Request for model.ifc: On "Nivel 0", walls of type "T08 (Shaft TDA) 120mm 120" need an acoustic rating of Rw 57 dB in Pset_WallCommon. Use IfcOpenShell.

First a look at what the model holds.

```python
import ifcopenshell
import ifcopenshell.util.element

model = ifcopenshell.open("model.ifc")
print(model.schema)
storey = next(s for s in model.by_type("IfcBuildingStorey") if s.Name == "Nivel 0")
walls = [e for e in ifcopenshell.util.element.get_decomposition(storey) if e.is_a("IfcWall")]
seen = {}
for e in walls:
    element_type = ifcopenshell.util.element.get_type(e)
    key = (element_type.Name if element_type != e and element_type else None, ifcopenshell.util.element.get_pset(e, "Pset_WallCommon", "AcousticRating"))
    seen[key] = seen.get(key, 0) + 1
for (name, value), count in sorted(seen.items(), key=str):
    print(count, "x", name, "|", value)
```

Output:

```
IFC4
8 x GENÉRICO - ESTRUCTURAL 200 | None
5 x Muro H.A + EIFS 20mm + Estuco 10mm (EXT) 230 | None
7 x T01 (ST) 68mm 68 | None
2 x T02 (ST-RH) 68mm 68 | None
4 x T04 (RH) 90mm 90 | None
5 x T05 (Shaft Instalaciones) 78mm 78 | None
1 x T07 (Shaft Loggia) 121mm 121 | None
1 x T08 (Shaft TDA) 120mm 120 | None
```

```python
import ifcopenshell
import ifcopenshell.api.pset
import ifcopenshell.util.element

model = ifcopenshell.open("model.ifc")

storey = next(s for s in model.by_type("IfcBuildingStorey") if s.Name == "Nivel 0")
walls = [e for e in ifcopenshell.util.element.get_decomposition(storey) if e.is_a("IfcWall")]

count = 0
for e in walls:
    element_type = ifcopenshell.util.element.get_type(e)
    if element_type in (None, e) or element_type.Name != "T08 (Shaft TDA) 120mm 120":
        continue
    # add_pset returns the element's existing set when there is one.
    pset = ifcopenshell.api.pset.add_pset(model, product=e, name="Pset_WallCommon")
    ifcopenshell.api.pset.edit_pset(model, pset=pset, properties={"AcousticRating": "Rw 57 dB"})
    count += 1

print(count, "walls updated")

model.write("model-out.ifc")
```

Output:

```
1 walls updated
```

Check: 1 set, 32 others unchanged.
